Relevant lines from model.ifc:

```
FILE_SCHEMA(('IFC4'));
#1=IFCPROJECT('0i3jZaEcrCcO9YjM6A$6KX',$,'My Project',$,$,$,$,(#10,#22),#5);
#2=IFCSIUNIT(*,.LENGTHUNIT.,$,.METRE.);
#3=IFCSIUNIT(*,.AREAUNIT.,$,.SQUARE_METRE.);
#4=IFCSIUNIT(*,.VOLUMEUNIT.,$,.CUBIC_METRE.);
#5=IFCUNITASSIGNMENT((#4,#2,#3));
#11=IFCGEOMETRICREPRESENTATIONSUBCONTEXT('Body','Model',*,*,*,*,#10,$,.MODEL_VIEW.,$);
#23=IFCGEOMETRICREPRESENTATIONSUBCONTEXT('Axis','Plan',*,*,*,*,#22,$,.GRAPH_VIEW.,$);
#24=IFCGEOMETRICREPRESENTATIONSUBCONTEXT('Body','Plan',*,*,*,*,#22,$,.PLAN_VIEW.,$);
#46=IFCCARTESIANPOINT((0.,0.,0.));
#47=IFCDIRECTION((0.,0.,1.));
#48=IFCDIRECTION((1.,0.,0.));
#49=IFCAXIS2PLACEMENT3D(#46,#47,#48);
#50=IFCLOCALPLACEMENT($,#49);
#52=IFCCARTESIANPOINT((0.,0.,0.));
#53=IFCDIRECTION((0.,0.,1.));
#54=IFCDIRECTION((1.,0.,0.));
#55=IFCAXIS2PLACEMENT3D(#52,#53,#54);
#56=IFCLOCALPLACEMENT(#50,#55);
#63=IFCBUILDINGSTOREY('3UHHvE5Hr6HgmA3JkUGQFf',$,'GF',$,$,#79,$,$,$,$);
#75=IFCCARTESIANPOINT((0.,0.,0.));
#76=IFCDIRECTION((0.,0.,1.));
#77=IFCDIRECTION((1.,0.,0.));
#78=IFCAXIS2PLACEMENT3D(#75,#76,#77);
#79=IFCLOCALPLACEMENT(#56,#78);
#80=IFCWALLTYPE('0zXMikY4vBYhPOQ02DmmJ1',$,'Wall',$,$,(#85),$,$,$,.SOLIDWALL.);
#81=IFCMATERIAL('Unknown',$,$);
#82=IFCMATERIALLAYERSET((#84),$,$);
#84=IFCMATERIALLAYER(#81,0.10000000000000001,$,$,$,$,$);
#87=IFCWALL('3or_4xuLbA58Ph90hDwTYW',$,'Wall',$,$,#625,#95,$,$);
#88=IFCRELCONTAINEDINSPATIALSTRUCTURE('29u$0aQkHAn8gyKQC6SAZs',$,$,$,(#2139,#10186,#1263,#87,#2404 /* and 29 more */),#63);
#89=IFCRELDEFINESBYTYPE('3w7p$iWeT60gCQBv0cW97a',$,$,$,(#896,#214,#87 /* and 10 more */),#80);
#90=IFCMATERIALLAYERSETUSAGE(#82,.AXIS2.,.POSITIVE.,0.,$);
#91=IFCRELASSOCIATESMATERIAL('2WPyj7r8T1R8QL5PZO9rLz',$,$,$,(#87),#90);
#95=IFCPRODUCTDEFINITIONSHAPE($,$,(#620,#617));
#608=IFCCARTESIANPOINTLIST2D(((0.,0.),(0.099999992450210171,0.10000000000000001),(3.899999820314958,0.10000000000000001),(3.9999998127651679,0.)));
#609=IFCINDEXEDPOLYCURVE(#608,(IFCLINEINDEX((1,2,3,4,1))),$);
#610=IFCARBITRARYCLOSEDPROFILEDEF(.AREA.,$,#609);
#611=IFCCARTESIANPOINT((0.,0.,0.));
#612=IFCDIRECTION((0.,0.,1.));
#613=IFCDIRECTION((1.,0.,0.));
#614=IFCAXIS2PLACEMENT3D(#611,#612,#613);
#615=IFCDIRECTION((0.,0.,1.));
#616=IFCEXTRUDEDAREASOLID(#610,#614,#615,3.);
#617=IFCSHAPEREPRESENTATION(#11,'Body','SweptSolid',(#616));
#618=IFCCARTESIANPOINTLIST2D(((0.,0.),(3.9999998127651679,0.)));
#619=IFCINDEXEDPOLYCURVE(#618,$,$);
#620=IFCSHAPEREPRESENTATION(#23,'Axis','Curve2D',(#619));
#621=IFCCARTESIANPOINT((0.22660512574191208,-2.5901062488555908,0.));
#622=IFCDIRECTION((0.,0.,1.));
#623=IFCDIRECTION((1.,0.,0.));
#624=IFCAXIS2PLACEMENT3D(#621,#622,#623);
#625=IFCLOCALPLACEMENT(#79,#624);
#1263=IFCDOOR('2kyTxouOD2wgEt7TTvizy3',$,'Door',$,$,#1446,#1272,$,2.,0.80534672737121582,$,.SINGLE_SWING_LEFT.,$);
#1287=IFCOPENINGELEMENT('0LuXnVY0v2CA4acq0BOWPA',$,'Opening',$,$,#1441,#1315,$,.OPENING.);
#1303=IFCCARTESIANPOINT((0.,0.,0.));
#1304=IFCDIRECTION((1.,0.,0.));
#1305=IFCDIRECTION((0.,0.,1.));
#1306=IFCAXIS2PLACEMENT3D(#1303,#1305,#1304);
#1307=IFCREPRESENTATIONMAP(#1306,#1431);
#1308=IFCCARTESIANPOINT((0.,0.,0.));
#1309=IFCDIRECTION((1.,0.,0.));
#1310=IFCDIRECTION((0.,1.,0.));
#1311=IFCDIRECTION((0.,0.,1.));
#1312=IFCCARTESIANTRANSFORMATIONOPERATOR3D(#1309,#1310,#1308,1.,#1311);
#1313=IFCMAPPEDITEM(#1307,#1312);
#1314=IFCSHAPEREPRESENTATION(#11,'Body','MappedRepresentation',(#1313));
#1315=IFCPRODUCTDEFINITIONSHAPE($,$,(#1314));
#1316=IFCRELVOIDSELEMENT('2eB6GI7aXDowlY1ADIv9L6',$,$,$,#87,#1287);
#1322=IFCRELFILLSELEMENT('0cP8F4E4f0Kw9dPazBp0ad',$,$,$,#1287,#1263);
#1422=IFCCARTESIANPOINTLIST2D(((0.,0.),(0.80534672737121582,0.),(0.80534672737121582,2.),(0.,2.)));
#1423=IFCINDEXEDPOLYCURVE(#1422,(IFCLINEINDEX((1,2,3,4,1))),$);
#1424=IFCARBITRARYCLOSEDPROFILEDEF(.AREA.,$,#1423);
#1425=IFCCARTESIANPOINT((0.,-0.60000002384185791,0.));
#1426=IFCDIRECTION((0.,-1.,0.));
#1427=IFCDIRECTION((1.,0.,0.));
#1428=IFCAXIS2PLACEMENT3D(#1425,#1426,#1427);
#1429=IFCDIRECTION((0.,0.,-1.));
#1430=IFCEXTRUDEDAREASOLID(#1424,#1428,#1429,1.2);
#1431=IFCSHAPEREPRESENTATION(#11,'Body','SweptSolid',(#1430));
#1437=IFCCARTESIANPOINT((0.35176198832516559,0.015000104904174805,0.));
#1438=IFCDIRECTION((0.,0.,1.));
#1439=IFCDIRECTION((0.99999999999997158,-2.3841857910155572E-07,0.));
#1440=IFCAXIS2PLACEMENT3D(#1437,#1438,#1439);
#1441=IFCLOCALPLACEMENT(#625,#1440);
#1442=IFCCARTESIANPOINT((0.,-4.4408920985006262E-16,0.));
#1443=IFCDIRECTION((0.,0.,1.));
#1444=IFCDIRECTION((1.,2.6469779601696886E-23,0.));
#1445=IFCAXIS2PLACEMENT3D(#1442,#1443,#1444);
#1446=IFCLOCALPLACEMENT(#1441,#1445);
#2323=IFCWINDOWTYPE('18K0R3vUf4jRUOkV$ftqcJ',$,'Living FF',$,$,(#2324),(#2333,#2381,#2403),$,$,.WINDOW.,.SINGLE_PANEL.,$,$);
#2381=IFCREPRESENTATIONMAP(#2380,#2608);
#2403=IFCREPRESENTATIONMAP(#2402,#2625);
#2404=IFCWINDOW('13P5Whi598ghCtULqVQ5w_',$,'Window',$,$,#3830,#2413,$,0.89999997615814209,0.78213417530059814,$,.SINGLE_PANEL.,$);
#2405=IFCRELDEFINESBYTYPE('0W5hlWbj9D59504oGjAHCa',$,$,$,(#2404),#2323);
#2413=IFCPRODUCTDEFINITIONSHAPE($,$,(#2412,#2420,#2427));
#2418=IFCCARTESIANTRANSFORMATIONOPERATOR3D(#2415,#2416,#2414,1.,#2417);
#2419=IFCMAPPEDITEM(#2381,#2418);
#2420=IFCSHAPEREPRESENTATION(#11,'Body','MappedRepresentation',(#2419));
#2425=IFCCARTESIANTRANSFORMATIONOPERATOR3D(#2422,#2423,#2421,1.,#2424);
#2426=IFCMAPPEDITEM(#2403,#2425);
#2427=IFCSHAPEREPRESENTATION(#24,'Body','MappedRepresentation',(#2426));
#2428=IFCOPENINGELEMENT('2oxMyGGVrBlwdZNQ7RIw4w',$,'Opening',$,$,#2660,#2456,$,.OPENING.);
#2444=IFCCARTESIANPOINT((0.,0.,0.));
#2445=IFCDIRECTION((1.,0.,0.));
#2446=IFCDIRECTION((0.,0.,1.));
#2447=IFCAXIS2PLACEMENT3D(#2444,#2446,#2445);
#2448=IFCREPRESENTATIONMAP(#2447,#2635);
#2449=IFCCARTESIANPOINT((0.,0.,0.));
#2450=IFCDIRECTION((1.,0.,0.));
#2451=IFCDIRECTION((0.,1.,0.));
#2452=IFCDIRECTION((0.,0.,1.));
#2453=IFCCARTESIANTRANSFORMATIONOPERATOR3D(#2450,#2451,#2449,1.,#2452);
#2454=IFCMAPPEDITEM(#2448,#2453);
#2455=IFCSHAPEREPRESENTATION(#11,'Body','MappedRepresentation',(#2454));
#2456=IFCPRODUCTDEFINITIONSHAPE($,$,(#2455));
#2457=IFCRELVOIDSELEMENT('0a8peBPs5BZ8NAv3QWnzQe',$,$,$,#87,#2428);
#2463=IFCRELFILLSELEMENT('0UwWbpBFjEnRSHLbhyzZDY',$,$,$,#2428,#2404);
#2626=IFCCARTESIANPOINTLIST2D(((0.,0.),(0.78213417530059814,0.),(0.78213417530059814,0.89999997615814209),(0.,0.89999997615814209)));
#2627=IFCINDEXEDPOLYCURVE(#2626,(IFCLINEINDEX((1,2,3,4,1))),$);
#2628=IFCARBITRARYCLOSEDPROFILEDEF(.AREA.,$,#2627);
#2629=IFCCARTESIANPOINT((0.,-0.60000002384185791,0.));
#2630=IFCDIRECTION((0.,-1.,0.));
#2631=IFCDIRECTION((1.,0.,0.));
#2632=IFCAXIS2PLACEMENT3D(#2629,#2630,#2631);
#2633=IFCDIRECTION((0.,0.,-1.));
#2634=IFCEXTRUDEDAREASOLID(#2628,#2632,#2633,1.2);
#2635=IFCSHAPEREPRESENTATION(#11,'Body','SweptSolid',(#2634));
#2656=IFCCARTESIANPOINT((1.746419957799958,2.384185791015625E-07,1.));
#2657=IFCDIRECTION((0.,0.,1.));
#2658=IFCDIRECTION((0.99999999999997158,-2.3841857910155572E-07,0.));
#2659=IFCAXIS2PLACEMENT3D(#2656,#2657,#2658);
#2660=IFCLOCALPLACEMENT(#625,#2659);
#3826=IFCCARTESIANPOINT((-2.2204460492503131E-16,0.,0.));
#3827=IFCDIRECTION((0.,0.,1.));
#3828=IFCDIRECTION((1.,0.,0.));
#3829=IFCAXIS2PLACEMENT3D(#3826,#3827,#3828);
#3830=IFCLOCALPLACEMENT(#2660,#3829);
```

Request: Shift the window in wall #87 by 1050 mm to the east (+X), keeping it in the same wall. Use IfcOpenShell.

```python
import ifcopenshell
import ifcopenshell.api.geometry
import ifcopenshell.util.placement

model = ifcopenshell.open("model.ifc")

window = model.by_guid("13P5Whi598ghCtULqVQ5w_")
opening = window.FillsVoids[0].RelatingOpeningElement
wall = opening.VoidsElements[0].RelatingBuildingElement

wall_matrix = ifcopenshell.util.placement.get_local_placement(wall.ObjectPlacement)
shift = wall_matrix[:3, 0] * 1.05
before = ifcopenshell.util.placement.get_local_placement(window.ObjectPlacement)[:3, 3].copy()

# The window is placed relative to its opening, so it follows when the opening moves.
matrix = ifcopenshell.util.placement.get_local_placement(opening.ObjectPlacement)
matrix[:3, 3] += shift
ifcopenshell.api.geometry.edit_object_placement(
    model, product=opening, matrix=matrix, is_si=False, should_transform_children=True
)

after = ifcopenshell.util.placement.get_local_placement(window.ObjectPlacement)[:3, 3]
print("window moved by", (after - before).round(3) + 0.0)

model.write("model-out.ifc")
```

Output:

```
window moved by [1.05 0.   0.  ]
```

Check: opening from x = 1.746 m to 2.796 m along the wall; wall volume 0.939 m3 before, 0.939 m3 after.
